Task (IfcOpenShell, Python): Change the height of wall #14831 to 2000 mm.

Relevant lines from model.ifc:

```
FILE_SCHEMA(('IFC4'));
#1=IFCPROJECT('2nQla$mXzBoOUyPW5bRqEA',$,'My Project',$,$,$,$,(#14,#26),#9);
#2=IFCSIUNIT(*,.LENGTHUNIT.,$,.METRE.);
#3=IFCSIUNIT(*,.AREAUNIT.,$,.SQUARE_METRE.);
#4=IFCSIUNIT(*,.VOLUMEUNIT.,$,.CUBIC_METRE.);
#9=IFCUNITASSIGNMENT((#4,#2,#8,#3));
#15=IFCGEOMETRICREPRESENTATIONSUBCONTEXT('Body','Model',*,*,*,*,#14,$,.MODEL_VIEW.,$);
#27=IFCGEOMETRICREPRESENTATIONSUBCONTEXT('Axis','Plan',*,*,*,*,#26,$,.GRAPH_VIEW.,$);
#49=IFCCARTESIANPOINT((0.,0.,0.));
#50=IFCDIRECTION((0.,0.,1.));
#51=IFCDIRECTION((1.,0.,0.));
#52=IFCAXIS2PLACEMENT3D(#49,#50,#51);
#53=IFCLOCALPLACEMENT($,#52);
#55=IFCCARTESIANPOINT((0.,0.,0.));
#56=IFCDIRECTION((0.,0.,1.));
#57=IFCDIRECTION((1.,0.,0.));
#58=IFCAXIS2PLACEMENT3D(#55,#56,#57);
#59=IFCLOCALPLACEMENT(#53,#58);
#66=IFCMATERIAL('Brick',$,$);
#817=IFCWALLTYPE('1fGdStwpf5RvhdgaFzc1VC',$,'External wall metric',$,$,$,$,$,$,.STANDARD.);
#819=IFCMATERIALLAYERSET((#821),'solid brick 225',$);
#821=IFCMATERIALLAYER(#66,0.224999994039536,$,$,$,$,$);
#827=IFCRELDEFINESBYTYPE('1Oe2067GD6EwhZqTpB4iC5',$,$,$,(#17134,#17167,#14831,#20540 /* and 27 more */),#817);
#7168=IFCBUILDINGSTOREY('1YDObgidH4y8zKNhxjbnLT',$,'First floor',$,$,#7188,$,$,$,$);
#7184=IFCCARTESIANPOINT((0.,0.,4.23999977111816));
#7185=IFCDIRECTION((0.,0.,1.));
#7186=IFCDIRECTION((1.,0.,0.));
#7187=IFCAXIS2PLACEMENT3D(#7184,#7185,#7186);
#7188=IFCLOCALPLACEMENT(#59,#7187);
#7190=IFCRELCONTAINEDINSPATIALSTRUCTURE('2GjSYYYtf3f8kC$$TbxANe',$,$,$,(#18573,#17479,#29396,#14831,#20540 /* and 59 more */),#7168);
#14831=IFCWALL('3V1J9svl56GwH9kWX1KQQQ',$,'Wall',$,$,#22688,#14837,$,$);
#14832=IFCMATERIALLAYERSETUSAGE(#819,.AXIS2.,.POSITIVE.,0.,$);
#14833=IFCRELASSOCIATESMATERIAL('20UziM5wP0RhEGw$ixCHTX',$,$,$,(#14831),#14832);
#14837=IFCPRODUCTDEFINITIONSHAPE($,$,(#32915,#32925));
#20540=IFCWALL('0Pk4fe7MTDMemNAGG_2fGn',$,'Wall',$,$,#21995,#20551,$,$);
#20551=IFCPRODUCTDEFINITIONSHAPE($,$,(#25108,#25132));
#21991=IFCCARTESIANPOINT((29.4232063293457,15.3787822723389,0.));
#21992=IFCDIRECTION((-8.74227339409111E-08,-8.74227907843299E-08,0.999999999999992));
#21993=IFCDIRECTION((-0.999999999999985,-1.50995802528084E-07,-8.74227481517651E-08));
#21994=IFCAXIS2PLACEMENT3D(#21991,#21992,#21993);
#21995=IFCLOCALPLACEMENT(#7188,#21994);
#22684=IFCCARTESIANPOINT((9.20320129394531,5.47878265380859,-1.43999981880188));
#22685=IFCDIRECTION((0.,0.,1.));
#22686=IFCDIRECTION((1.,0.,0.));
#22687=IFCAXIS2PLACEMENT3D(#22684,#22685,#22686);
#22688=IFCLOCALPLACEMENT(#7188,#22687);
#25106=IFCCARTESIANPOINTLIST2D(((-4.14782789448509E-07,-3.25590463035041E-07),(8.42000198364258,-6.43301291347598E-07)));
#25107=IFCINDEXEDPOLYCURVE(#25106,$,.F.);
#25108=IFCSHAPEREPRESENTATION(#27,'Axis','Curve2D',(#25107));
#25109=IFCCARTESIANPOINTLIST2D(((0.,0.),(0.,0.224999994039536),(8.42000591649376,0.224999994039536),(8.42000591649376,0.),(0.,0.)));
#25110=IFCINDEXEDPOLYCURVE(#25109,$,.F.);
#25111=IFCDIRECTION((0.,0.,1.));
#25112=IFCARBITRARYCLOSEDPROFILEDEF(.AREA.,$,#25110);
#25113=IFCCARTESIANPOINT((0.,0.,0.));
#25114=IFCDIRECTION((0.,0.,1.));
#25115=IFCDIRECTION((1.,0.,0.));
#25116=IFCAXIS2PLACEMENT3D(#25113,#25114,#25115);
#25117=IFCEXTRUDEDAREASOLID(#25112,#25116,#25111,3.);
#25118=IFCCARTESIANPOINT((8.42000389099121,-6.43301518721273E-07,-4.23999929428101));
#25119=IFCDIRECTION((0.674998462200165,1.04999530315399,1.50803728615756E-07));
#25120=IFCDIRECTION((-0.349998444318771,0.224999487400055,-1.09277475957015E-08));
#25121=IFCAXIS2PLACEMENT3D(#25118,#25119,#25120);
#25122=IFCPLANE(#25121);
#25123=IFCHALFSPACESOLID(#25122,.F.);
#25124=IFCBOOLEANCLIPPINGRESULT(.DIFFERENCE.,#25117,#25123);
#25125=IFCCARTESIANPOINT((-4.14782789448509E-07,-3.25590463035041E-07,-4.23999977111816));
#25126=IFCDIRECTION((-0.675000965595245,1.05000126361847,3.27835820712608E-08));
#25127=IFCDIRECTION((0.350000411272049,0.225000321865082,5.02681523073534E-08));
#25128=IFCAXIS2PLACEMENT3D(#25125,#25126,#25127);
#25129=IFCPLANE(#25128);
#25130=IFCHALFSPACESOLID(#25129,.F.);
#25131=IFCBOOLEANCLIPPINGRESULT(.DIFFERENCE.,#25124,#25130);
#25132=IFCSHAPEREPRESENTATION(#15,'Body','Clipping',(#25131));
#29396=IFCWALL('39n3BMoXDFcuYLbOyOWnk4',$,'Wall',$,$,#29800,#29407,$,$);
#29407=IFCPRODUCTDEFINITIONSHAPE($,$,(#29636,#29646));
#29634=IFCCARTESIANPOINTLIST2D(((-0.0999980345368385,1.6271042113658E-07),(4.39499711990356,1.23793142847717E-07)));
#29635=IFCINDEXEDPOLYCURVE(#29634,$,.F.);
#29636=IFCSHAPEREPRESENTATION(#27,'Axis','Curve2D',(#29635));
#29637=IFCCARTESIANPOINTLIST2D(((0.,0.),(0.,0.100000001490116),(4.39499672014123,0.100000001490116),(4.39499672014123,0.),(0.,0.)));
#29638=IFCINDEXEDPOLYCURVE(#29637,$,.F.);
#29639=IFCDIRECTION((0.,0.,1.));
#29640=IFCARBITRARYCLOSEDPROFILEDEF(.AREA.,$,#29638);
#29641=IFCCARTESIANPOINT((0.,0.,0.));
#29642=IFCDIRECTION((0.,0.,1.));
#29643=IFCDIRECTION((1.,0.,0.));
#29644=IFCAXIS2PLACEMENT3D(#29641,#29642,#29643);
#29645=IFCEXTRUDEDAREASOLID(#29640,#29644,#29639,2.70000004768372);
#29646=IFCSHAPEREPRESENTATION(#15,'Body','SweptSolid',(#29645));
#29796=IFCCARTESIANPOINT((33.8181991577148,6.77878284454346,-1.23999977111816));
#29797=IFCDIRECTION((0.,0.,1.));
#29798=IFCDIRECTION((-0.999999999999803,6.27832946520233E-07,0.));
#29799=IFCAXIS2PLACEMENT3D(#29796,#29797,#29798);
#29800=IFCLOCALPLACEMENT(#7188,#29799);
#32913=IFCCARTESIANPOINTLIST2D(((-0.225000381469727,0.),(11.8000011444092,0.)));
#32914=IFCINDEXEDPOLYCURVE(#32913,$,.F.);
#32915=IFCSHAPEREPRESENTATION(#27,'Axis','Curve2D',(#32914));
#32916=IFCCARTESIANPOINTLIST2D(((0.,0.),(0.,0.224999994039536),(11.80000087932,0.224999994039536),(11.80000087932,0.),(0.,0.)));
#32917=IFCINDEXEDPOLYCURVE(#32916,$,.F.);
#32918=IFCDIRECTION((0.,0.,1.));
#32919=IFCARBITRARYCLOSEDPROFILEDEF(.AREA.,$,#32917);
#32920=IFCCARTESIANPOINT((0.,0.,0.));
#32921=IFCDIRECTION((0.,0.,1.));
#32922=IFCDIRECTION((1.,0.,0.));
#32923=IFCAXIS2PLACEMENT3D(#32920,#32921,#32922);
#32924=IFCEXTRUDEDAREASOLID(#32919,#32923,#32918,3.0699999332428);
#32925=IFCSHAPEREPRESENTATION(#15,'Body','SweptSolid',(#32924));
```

```python
import ifcopenshell
import ifcopenshell.geom
import ifcopenshell.util.representation
import ifcopenshell.util.shape

model = ifcopenshell.open("model.ifc")
settings = ifcopenshell.geom.settings()


def volume(element):
    """Net volume in cubic metres, openings subtracted."""
    shape = ifcopenshell.geom.create_shape(settings, element)
    return ifcopenshell.util.shape.get_volume(shape.geometry)


wall = model.by_id(14831)
before = volume(wall)

body = ifcopenshell.util.representation.get_representation(wall, "Model", "Body")
solid = body.Items[0]
old_height = solid.Depth
solid.Depth = 2.0
after = volume(wall)

print(f"height {old_height:g} -> {solid.Depth:g}, volume {before:.3f} -> {after:.3f} m3")

model.write("model_v2.ifc")
```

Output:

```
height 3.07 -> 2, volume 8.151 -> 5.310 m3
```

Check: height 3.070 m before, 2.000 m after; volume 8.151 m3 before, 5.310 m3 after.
